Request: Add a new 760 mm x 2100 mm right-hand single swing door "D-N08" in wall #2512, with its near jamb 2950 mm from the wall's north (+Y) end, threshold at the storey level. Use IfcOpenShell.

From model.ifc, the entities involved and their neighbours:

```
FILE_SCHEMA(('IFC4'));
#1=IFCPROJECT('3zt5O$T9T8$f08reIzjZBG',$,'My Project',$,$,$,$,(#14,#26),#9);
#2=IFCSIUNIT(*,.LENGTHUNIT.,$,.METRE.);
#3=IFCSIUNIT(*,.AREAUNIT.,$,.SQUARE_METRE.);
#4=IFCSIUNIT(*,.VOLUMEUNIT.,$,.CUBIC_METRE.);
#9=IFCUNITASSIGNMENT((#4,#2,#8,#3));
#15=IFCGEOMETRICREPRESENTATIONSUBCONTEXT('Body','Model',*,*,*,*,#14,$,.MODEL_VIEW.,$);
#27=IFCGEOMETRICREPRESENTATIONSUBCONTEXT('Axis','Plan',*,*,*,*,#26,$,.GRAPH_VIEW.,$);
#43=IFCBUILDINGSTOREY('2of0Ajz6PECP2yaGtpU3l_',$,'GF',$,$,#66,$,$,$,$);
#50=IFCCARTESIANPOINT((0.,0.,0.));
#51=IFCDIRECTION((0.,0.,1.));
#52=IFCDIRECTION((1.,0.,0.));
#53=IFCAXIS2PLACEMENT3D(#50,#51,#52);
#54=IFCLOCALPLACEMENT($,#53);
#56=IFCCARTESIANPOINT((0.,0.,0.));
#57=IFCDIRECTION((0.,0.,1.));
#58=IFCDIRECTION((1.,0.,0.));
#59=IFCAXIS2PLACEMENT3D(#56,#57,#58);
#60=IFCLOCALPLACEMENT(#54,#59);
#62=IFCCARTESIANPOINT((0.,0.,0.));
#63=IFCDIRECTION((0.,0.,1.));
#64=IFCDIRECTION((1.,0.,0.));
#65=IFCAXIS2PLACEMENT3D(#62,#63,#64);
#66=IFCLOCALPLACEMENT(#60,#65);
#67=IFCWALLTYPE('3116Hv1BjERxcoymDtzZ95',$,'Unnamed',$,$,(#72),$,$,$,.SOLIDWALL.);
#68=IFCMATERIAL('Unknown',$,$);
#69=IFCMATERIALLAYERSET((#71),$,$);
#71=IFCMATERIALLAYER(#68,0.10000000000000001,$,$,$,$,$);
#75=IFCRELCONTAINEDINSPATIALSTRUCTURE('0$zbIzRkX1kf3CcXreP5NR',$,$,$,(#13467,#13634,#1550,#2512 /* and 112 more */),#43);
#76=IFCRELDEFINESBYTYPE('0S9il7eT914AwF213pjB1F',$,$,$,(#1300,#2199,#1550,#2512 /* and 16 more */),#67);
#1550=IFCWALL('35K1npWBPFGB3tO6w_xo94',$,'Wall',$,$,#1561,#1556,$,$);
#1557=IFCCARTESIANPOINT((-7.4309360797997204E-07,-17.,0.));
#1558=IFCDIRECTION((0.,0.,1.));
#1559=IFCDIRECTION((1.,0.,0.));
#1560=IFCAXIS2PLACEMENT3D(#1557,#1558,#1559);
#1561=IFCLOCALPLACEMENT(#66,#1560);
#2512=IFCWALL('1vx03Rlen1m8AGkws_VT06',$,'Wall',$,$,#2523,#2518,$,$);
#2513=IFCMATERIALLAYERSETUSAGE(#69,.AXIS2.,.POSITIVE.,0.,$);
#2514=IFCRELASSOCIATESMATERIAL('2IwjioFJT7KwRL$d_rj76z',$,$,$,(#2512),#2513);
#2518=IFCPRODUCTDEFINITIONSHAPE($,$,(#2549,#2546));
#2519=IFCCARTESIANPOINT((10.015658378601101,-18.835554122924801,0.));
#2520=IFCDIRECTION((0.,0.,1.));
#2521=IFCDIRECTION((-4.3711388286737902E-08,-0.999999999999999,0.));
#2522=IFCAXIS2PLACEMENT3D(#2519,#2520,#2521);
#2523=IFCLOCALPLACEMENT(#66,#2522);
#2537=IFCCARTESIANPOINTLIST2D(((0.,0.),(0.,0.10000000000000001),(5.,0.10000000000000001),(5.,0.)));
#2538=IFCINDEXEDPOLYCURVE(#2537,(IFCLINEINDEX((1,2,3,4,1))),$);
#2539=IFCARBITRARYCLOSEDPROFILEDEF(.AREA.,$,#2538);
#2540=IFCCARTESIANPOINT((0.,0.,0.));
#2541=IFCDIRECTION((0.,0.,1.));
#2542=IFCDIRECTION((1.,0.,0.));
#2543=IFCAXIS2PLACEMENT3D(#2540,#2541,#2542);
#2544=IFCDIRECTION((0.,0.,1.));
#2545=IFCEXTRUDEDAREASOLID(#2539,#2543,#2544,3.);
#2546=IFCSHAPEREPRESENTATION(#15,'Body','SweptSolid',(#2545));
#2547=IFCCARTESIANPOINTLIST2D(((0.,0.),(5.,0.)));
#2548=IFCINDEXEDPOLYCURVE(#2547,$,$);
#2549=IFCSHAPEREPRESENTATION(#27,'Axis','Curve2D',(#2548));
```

```python
import numpy as np
import ifcopenshell
import ifcopenshell.api.feature
import ifcopenshell.api.geometry
import ifcopenshell.api.root
import ifcopenshell.api.spatial
import ifcopenshell.geom
import ifcopenshell.util.element
import ifcopenshell.util.placement
import ifcopenshell.util.representation
import ifcopenshell.util.shape
import ifcopenshell.util.unit

model = ifcopenshell.open("model.ifc")
unit_scale = ifcopenshell.util.unit.calculate_unit_scale(model)
settings = ifcopenshell.geom.settings()


def volume(element):
    """Net volume in cubic metres, openings subtracted."""
    shape = ifcopenshell.geom.create_shape(settings, element)
    return ifcopenshell.util.shape.get_volume(shape.geometry)


wall = model.by_guid("1vx03Rlen1m8AGkws_VT06")
storey = ifcopenshell.util.element.get_container(wall, ifc_class="IfcBuildingStorey")
context = ifcopenshell.util.representation.get_context(model, "Model", "Body", "MODEL_VIEW")
before = volume(wall)

width, height, from_end, sill = 0.76, 2.1, 2.95, 0.0  # metres

# The wall runs along its own X axis, and the end named is its -X end.
wall_shape = ifcopenshell.geom.create_shape(settings, wall)
x, y, z = ifcopenshell.util.shape.get_vertices(wall_shape.geometry).T
start = x.min() + from_end
face, thickness = float(y.min()), float(y.max() - y.min())
wall_matrix = ifcopenshell.util.placement.get_local_placement(wall.ObjectPlacement)
level = ifcopenshell.util.placement.get_local_placement(storey.ObjectPlacement)[2, 3]


def in_wall(x, y):
    """Placement at x, y metres in the wall's axes, at sill height."""
    matrix = wall_matrix.copy()
    matrix[:, 3] = wall_matrix @ np.array([x / unit_scale, y / unit_scale, 0.0, 1.0])
    matrix[2, 3] = level + sill / unit_scale
    return matrix


# Opening: a box that overshoots both wall faces by 50 mm.
opening = ifcopenshell.api.root.create_entity(model, ifc_class="IfcOpeningElement", predefined_type="OPENING")
box = ifcopenshell.api.geometry.add_wall_representation(
    model, context=context, length=width, height=height, thickness=thickness + 0.1
)
ifcopenshell.api.geometry.assign_representation(model, product=opening, representation=box)
ifcopenshell.api.geometry.edit_object_placement(model, product=opening, matrix=in_wall(start, face - 0.05), is_si=False)
ifcopenshell.api.feature.add_feature(model, feature=opening, element=wall)

door = ifcopenshell.api.root.create_entity(model, ifc_class="IfcDoor", name="D-N08", predefined_type="DOOR")
door.OverallWidth, door.OverallHeight = width / unit_scale, height / unit_scale
door.OperationType = "SINGLE_SWING_RIGHT"
body = ifcopenshell.api.geometry.add_door_representation(
    model,
    context=context,
    overall_width=door.OverallWidth,
    overall_height=door.OverallHeight,
    operation_type="SINGLE_SWING_RIGHT",
    lining_properties={"LiningDepth": thickness / unit_scale, "ThresholdDepth": thickness / unit_scale},
)
ifcopenshell.api.geometry.assign_representation(model, product=door, representation=body)
ifcopenshell.api.spatial.assign_container(model, products=[door], relating_structure=storey)
ifcopenshell.api.feature.add_filling(model, opening=opening, element=door)

# The lining spans the wall, so the door starts at the wall face.
ifcopenshell.api.geometry.edit_object_placement(model, product=door, matrix=in_wall(start, face), is_si=False)

after = volume(wall)

print(f"wall volume {before:.3f} -> {after:.3f} m3")

model.write("model_rev.ifc")
```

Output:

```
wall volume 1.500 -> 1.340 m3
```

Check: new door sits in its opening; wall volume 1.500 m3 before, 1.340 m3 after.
